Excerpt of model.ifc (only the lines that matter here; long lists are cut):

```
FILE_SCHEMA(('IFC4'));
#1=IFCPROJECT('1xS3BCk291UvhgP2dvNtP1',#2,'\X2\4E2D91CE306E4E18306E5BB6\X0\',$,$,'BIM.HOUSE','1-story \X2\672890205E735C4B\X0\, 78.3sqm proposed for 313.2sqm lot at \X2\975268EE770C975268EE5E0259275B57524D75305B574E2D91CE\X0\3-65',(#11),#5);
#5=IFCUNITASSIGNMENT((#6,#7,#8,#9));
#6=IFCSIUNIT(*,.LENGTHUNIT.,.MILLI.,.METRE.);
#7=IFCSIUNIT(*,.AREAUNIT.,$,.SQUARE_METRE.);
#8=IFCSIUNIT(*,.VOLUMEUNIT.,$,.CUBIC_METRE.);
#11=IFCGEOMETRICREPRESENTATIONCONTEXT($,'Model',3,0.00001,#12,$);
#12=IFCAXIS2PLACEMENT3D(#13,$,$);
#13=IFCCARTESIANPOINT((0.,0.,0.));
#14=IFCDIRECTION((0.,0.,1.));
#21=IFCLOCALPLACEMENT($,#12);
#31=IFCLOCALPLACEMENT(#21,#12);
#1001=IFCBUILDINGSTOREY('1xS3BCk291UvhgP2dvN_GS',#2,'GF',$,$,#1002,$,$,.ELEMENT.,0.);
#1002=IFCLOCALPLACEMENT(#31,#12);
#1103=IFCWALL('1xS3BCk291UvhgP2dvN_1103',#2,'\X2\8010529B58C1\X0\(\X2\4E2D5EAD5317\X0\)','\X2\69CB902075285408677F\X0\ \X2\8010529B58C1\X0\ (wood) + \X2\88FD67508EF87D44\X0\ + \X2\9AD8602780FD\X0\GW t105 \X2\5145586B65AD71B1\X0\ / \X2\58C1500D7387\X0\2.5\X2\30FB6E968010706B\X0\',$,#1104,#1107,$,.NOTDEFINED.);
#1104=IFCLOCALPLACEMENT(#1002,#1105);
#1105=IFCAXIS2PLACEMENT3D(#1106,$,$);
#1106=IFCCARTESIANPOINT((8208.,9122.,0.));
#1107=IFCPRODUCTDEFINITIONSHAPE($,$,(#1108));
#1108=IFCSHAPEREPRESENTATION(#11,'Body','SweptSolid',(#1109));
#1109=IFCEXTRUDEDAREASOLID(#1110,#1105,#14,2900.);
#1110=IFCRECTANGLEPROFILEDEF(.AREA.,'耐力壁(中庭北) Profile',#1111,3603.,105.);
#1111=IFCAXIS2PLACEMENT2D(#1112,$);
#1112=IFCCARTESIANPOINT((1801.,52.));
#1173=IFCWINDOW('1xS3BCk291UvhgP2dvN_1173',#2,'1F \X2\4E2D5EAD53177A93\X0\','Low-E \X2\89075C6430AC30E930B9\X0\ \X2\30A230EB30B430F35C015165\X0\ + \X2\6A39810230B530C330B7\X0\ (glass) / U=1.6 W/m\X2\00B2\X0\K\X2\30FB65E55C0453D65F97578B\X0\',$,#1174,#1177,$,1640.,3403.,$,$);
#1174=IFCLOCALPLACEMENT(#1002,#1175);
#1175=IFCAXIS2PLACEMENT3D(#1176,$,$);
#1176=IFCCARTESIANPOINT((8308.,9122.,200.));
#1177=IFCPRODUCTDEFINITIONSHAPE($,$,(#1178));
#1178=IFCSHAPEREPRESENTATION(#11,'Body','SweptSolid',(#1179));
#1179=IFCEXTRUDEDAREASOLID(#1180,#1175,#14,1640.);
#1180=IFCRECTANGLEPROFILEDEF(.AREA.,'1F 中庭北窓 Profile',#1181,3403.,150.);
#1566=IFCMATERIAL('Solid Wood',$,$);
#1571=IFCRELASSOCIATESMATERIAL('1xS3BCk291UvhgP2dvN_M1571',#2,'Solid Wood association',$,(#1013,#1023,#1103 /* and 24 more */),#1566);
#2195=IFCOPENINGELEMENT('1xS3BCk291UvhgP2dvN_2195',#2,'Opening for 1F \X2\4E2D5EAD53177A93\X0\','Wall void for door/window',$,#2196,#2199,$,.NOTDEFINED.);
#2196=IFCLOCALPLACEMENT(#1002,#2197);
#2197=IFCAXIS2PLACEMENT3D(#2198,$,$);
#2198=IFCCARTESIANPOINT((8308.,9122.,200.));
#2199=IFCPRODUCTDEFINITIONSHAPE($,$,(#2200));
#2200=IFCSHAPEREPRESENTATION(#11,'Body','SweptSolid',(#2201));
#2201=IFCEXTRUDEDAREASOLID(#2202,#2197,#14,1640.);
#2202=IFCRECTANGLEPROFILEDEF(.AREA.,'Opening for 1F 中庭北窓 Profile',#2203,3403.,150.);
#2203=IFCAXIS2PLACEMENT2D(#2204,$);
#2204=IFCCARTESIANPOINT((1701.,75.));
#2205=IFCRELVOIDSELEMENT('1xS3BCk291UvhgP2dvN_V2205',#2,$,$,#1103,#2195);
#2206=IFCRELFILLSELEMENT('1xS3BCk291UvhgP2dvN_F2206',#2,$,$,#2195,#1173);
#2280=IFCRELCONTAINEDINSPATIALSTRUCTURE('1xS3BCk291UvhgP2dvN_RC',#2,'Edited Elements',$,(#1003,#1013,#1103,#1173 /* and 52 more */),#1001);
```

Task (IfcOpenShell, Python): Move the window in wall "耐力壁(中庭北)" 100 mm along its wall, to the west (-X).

```python
import ifcopenshell
import ifcopenshell.api.geometry
import ifcopenshell.util.placement
import ifcopenshell.util.unit

model = ifcopenshell.open("model.ifc")
unit_scale = ifcopenshell.util.unit.calculate_unit_scale(model)

window = model.by_id(1173)
opening = window.FillsVoids[0].RelatingOpeningElement
wall = opening.VoidsElements[0].RelatingBuildingElement

wall_matrix = ifcopenshell.util.placement.get_local_placement(wall.ObjectPlacement)
shift = wall_matrix[:3, 0] * -0.1 / unit_scale
before = ifcopenshell.util.placement.get_local_placement(window.ObjectPlacement)[:3, 3].copy()

# The window is not placed relative to its opening, so move both.
for product in (opening, window):
    matrix = ifcopenshell.util.placement.get_local_placement(product.ObjectPlacement)
    matrix[:3, 3] += shift
    ifcopenshell.api.geometry.edit_object_placement(model, product=product, matrix=matrix, is_si=False)

after = ifcopenshell.util.placement.get_local_placement(window.ObjectPlacement)[:3, 3]
print("window moved by", (after - before).round(3) + 0.0)

model.write("model_edited.ifc")
```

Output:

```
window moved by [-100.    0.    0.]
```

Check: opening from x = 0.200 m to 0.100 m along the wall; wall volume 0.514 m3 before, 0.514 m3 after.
